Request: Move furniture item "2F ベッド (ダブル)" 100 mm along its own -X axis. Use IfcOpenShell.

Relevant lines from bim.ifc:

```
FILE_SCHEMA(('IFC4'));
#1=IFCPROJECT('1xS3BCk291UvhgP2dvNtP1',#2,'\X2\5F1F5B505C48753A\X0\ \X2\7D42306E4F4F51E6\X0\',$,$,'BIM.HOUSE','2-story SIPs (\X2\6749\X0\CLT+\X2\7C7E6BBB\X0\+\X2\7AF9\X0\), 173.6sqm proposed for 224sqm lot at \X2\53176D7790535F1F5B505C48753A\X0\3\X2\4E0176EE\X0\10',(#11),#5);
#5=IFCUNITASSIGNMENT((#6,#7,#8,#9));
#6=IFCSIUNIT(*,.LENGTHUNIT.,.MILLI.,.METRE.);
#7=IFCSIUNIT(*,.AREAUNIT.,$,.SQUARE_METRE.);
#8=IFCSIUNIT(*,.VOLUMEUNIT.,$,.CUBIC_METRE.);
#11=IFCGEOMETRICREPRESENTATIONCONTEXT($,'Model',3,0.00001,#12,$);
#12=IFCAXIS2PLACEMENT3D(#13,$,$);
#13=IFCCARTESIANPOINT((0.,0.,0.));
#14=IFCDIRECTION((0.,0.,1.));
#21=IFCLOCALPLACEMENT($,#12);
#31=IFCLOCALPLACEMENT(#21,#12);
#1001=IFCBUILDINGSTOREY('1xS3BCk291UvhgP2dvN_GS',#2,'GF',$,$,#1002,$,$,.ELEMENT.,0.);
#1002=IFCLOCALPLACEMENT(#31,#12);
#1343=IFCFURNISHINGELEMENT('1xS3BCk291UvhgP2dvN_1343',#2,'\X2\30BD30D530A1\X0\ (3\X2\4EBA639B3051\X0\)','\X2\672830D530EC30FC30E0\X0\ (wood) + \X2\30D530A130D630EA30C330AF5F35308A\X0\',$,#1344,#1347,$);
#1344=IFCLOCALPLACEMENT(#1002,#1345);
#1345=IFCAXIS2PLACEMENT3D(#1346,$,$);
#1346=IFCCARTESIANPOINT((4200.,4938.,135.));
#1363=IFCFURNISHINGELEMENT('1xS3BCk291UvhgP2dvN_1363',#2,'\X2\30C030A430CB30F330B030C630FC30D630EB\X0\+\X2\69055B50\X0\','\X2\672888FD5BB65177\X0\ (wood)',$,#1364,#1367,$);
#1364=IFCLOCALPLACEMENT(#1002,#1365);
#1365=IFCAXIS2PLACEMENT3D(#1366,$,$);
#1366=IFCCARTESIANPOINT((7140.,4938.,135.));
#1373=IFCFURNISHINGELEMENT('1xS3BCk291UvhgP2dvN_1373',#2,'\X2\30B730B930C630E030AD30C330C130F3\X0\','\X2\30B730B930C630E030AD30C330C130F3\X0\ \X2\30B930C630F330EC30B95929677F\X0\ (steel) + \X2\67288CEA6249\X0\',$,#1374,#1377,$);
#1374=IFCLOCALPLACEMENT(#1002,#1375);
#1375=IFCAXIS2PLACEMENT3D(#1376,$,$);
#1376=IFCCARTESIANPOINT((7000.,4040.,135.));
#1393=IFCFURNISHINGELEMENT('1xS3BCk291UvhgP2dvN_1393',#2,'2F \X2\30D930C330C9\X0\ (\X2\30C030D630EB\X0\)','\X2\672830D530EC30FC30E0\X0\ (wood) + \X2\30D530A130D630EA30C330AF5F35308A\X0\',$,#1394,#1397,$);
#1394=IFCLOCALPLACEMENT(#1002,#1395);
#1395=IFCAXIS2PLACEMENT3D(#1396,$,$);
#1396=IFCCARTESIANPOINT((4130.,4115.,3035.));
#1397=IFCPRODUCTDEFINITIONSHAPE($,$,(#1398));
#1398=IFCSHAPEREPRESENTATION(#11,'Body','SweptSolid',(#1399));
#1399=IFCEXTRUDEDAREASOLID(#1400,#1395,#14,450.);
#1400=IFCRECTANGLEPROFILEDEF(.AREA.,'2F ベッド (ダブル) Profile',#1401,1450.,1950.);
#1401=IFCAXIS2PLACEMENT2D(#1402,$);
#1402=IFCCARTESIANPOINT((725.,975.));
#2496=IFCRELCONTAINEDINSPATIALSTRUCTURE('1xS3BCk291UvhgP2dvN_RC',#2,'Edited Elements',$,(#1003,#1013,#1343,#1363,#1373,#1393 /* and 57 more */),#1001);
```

```python
import ifcopenshell
import ifcopenshell.api.geometry
import ifcopenshell.util.placement
import ifcopenshell.util.unit

model = ifcopenshell.open("bim.ifc")
unit_scale = ifcopenshell.util.unit.calculate_unit_scale(model)

item = model.by_guid("1xS3BCk291UvhgP2dvN_1393")
matrix = ifcopenshell.util.placement.get_local_placement(item.ObjectPlacement)
matrix[:3, 3] -= matrix[:3, 0] * 0.1 / unit_scale
ifcopenshell.api.geometry.edit_object_placement(model, product=item, matrix=matrix, is_si=False)

print(ifcopenshell.util.placement.get_local_placement(item.ObjectPlacement).round(3) + 0.0)

model.write("bim_edited.ifc")
```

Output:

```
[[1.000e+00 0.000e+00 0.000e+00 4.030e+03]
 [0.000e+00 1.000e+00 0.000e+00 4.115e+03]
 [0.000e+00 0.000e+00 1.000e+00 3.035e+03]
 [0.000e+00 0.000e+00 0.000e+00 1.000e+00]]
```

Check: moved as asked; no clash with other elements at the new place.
